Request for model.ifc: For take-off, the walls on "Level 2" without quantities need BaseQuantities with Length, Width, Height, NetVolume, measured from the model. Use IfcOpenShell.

First a look at what the model holds.

```python
import ifcopenshell
import ifcopenshell.util.element
import ifcopenshell.util.unit

model = ifcopenshell.open("model.ifc")
print(model.schema)
for unit_type in ("LENGTHUNIT", "AREAUNIT", "VOLUMEUNIT"):
    print(unit_type, ifcopenshell.util.unit.calculate_unit_scale(model, unit_type))
storey = next(s for s in model.by_type("IfcBuildingStorey") if s.Name == "Level 2")
walls = [e for e in ifcopenshell.util.element.get_decomposition(storey) if e.is_a("IfcWall")]
for e in sorted(walls, key=lambda e: e.id()):
    print(e.id(), e.is_a(), e.Name, list(ifcopenshell.util.element.get_psets(e, qtos_only=True)), sep=" | ")
```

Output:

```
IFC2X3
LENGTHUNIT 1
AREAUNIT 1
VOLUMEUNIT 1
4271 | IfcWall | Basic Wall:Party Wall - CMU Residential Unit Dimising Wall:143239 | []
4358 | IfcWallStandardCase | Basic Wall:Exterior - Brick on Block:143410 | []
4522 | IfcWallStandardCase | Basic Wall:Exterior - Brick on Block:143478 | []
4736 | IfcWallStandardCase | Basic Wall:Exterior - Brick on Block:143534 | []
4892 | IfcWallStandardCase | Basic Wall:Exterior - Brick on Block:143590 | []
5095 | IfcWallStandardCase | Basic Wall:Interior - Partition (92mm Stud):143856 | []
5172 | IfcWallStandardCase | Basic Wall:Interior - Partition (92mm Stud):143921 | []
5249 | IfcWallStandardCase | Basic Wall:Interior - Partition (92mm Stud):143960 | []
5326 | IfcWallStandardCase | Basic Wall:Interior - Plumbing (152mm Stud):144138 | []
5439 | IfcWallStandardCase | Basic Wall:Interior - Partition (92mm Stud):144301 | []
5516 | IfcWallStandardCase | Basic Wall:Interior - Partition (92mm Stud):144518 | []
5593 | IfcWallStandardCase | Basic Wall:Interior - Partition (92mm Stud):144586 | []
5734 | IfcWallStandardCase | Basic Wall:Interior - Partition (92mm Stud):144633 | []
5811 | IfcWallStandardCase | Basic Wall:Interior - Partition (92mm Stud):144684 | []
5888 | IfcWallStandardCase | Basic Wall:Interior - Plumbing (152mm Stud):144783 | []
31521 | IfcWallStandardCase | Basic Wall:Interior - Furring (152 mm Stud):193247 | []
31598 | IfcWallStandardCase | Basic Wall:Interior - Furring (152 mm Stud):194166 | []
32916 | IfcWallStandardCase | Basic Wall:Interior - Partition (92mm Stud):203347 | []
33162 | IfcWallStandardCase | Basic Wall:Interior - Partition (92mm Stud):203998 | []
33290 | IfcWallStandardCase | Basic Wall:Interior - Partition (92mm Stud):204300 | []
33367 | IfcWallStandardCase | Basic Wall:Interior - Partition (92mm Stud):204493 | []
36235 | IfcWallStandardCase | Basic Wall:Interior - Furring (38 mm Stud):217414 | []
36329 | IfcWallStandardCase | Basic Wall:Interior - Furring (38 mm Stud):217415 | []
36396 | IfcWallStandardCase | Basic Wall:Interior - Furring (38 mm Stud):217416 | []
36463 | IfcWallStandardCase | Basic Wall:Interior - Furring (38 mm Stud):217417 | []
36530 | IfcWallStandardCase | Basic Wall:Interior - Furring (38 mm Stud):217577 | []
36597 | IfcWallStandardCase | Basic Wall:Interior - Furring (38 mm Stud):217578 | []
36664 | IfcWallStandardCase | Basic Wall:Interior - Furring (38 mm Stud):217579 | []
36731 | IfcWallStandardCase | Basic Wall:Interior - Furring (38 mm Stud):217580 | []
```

```python
import ifcopenshell
import ifcopenshell.api.pset
import ifcopenshell.geom
import ifcopenshell.util.element
import ifcopenshell.util.shape
import ifcopenshell.util.unit

model = ifcopenshell.open("model.ifc")
unit_scale = ifcopenshell.util.unit.calculate_unit_scale(model)
volume_scale = ifcopenshell.util.unit.calculate_unit_scale(model, "VOLUMEUNIT")
settings = ifcopenshell.geom.settings()

storey = next(s for s in model.by_type("IfcBuildingStorey") if s.Name == "Level 2")
walls = [e for e in ifcopenshell.util.element.get_decomposition(storey) if e.is_a("IfcWall")]

for e in sorted(walls, key=lambda e: e.id()):
    if ifcopenshell.util.element.get_psets(e, qtos_only=True, should_inherit=False):
        continue
    # Geometry comes back in metres, in the element's own axes.
    shape = ifcopenshell.geom.create_shape(settings, e)
    values = {
        "Length": ifcopenshell.util.shape.get_x(shape.geometry) / unit_scale,
        "Width": ifcopenshell.util.shape.get_y(shape.geometry) / unit_scale,
        "Height": ifcopenshell.util.shape.get_z(shape.geometry) / unit_scale,
        "NetVolume": ifcopenshell.util.shape.get_volume(shape.geometry) / volume_scale,
    }
    qto = ifcopenshell.api.pset.add_qto(model, product=e, name="BaseQuantities")
    ifcopenshell.api.pset.edit_qto(model, qto=qto, properties=values)
    print(e.id(), {k: round(v, 3) for k, v in values.items()})

model.write("model_v2.ifc")
```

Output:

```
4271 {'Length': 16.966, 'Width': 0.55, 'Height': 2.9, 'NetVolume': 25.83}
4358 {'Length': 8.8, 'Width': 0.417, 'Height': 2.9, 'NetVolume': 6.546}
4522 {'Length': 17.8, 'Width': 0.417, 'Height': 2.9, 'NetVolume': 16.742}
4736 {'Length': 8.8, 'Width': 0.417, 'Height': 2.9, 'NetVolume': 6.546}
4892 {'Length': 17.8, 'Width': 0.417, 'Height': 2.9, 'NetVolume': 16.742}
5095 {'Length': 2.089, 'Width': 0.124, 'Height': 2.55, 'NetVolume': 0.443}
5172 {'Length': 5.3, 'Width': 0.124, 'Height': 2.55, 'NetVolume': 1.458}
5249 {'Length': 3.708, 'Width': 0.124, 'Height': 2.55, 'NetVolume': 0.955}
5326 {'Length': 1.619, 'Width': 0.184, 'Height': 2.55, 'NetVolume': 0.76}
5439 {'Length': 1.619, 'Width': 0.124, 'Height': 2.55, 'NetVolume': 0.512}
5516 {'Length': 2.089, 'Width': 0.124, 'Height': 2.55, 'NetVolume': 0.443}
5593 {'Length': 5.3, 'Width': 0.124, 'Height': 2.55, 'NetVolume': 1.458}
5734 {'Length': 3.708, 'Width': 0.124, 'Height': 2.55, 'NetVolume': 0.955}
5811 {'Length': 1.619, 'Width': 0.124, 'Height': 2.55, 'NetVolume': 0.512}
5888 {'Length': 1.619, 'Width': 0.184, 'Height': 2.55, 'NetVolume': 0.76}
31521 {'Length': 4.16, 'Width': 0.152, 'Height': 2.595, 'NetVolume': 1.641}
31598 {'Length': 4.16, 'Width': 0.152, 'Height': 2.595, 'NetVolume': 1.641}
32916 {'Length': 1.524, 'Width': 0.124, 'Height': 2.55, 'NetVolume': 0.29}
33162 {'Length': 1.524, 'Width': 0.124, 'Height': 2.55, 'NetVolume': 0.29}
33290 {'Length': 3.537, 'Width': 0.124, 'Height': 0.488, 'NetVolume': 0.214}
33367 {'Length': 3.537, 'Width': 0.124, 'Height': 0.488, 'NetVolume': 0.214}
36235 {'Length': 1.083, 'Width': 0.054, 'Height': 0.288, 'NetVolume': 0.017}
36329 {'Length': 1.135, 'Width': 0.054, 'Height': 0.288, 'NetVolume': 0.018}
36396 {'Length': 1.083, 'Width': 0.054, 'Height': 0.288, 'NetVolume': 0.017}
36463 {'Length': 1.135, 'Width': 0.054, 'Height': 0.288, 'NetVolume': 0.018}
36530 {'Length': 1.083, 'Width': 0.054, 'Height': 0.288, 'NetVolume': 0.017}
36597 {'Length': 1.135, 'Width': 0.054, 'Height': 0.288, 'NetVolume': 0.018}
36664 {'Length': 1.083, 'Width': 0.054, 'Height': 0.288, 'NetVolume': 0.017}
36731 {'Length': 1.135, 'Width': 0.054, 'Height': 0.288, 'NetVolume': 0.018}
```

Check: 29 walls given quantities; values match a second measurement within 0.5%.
